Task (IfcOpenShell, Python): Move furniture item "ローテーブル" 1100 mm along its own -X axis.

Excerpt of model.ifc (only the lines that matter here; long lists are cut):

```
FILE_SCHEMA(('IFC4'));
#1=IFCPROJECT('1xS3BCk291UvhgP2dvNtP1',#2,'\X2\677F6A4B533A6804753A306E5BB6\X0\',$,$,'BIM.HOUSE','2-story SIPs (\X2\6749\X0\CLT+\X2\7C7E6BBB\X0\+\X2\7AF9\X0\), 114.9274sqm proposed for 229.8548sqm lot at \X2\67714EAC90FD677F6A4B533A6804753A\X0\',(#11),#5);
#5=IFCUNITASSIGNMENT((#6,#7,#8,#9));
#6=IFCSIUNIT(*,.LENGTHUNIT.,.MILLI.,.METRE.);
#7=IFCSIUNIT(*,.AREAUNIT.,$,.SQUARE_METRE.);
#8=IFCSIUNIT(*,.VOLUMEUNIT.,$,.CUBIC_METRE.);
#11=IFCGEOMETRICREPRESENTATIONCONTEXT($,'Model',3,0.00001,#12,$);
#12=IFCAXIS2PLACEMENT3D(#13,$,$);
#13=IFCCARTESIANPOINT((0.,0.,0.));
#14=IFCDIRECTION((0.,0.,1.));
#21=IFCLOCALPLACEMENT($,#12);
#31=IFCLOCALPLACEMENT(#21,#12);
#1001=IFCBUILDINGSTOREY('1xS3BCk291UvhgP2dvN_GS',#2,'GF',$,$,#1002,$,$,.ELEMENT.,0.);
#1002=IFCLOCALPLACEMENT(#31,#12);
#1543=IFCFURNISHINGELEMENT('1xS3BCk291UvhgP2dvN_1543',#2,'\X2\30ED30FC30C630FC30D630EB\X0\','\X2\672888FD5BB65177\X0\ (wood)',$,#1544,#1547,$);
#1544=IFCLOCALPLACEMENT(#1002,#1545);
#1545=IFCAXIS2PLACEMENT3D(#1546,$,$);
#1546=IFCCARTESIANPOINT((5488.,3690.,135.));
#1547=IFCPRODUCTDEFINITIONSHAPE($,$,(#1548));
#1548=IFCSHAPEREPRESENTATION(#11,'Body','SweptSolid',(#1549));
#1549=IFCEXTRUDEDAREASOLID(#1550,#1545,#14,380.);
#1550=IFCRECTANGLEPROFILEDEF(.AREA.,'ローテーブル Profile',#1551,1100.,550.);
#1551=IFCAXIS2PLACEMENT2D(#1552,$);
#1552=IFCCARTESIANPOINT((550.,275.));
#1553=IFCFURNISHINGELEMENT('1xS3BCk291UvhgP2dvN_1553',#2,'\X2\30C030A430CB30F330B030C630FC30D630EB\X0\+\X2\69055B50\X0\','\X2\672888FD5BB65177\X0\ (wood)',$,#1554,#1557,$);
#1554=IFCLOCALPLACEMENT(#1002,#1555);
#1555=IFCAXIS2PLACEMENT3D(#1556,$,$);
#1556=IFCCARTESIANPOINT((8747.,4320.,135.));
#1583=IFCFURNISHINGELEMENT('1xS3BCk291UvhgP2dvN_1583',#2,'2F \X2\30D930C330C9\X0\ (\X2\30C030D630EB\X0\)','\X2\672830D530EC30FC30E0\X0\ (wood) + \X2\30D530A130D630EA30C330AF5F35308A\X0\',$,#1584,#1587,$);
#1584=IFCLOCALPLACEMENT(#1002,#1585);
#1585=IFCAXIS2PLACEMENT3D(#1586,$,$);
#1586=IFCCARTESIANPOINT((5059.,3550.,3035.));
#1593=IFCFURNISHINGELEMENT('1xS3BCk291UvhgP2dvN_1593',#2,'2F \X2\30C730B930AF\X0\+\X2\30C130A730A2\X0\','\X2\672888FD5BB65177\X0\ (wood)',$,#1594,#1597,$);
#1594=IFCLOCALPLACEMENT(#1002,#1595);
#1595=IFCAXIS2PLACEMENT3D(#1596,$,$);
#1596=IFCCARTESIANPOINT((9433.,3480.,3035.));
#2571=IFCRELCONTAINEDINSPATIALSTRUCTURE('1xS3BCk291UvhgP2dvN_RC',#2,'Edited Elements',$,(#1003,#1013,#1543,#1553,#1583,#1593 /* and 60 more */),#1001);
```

```python
import ifcopenshell
import ifcopenshell.api.geometry
import ifcopenshell.util.placement

model = ifcopenshell.open("model.ifc")

item = model.by_id(1543)
matrix = ifcopenshell.util.placement.get_local_placement(item.ObjectPlacement)
matrix[:3, 3] -= matrix[:3, 0] * 1100.0
ifcopenshell.api.geometry.edit_object_placement(model, product=item, matrix=matrix, is_si=False)

print(ifcopenshell.util.placement.get_local_placement(item.ObjectPlacement).round(3) + 0.0)

model.write("model_edited.ifc")
```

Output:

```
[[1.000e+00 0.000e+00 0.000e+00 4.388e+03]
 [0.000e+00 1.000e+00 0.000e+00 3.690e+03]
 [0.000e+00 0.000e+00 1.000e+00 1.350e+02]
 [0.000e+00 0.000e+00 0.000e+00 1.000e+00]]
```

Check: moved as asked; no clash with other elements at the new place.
